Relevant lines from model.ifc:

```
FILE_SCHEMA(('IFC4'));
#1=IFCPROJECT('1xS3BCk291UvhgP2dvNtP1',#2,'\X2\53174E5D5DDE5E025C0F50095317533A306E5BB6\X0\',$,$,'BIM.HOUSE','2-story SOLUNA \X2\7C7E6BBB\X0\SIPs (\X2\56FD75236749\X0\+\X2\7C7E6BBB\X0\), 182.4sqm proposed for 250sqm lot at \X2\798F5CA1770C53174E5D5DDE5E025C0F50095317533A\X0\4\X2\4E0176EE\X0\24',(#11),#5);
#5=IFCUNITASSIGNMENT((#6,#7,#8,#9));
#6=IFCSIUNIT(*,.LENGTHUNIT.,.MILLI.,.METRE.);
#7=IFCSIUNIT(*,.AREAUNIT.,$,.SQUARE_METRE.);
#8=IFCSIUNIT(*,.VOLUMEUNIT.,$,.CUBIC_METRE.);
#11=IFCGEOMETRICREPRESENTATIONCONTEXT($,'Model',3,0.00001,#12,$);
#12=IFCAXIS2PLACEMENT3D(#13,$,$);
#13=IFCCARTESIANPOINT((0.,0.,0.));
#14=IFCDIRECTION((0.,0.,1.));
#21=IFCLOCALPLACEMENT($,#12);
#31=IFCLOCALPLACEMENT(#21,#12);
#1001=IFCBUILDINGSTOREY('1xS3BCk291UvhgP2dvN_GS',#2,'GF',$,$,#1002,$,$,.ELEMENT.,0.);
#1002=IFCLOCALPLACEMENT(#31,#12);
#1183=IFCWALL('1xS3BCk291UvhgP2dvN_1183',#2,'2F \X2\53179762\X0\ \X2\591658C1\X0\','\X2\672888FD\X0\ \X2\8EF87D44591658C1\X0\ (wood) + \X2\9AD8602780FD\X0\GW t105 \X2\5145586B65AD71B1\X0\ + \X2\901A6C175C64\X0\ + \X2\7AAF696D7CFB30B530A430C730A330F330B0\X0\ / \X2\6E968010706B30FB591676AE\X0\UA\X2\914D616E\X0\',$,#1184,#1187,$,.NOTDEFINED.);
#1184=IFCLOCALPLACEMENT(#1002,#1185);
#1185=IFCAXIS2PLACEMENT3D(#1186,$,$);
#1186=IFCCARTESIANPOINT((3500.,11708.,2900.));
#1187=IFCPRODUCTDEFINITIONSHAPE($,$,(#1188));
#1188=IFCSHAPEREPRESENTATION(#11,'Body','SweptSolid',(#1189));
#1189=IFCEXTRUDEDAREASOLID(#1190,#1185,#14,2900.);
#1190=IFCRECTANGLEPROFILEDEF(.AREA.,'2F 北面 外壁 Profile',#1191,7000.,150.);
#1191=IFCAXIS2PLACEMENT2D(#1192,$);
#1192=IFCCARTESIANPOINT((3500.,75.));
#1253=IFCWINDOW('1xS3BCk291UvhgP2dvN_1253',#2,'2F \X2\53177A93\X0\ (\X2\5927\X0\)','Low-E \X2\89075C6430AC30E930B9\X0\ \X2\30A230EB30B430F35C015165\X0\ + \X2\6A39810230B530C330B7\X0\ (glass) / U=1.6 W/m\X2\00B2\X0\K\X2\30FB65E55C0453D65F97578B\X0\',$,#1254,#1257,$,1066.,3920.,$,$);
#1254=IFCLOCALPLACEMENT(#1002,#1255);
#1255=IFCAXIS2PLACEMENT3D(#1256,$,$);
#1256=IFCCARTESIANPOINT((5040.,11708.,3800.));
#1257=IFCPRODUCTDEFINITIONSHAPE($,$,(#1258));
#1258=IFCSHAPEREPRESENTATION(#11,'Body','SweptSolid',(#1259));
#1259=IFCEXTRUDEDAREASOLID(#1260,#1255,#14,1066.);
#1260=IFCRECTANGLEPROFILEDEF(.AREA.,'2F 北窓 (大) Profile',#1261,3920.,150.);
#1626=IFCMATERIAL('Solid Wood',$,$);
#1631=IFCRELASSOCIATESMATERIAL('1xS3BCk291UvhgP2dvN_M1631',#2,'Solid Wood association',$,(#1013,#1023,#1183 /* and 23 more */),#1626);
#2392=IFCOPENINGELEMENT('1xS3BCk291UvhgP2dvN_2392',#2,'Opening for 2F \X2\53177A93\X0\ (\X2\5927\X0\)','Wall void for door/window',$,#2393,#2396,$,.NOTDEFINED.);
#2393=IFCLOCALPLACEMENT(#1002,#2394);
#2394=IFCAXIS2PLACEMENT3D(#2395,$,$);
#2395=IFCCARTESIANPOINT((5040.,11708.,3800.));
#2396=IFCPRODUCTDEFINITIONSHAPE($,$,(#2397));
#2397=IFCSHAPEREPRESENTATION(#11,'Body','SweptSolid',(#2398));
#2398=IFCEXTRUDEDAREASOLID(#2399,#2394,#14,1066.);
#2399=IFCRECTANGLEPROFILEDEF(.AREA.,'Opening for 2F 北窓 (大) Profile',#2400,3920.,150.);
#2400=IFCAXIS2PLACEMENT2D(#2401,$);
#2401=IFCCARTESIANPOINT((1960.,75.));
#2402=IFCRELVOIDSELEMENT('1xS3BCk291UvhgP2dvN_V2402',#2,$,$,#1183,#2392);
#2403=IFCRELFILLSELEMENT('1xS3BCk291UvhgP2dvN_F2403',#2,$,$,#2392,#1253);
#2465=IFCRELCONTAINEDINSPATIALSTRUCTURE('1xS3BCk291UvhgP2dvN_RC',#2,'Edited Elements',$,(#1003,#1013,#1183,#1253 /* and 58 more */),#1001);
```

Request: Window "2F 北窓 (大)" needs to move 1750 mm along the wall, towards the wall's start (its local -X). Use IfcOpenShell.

```python
import ifcopenshell
import ifcopenshell.api.geometry
import ifcopenshell.util.placement
import ifcopenshell.util.unit

model = ifcopenshell.open("model.ifc")
unit_scale = ifcopenshell.util.unit.calculate_unit_scale(model)

window = model.by_id(1253)
opening = window.FillsVoids[0].RelatingOpeningElement
wall = opening.VoidsElements[0].RelatingBuildingElement

wall_matrix = ifcopenshell.util.placement.get_local_placement(wall.ObjectPlacement)
shift = wall_matrix[:3, 0] * -1.75 / unit_scale
before = ifcopenshell.util.placement.get_local_placement(window.ObjectPlacement)[:3, 3].copy()

# The window is not placed relative to its opening, so move both.
for product in (opening, window):
    matrix = ifcopenshell.util.placement.get_local_placement(product.ObjectPlacement)
    matrix[:3, 3] += shift
    ifcopenshell.api.geometry.edit_object_placement(model, product=product, matrix=matrix, is_si=False)

after = ifcopenshell.util.placement.get_local_placement(window.ObjectPlacement)[:3, 3]
print("window moved by", (after - before).round(3) + 0.0)

model.write("model_edited.ifc")
```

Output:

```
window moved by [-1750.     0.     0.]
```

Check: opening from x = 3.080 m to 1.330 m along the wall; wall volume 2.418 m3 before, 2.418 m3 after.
